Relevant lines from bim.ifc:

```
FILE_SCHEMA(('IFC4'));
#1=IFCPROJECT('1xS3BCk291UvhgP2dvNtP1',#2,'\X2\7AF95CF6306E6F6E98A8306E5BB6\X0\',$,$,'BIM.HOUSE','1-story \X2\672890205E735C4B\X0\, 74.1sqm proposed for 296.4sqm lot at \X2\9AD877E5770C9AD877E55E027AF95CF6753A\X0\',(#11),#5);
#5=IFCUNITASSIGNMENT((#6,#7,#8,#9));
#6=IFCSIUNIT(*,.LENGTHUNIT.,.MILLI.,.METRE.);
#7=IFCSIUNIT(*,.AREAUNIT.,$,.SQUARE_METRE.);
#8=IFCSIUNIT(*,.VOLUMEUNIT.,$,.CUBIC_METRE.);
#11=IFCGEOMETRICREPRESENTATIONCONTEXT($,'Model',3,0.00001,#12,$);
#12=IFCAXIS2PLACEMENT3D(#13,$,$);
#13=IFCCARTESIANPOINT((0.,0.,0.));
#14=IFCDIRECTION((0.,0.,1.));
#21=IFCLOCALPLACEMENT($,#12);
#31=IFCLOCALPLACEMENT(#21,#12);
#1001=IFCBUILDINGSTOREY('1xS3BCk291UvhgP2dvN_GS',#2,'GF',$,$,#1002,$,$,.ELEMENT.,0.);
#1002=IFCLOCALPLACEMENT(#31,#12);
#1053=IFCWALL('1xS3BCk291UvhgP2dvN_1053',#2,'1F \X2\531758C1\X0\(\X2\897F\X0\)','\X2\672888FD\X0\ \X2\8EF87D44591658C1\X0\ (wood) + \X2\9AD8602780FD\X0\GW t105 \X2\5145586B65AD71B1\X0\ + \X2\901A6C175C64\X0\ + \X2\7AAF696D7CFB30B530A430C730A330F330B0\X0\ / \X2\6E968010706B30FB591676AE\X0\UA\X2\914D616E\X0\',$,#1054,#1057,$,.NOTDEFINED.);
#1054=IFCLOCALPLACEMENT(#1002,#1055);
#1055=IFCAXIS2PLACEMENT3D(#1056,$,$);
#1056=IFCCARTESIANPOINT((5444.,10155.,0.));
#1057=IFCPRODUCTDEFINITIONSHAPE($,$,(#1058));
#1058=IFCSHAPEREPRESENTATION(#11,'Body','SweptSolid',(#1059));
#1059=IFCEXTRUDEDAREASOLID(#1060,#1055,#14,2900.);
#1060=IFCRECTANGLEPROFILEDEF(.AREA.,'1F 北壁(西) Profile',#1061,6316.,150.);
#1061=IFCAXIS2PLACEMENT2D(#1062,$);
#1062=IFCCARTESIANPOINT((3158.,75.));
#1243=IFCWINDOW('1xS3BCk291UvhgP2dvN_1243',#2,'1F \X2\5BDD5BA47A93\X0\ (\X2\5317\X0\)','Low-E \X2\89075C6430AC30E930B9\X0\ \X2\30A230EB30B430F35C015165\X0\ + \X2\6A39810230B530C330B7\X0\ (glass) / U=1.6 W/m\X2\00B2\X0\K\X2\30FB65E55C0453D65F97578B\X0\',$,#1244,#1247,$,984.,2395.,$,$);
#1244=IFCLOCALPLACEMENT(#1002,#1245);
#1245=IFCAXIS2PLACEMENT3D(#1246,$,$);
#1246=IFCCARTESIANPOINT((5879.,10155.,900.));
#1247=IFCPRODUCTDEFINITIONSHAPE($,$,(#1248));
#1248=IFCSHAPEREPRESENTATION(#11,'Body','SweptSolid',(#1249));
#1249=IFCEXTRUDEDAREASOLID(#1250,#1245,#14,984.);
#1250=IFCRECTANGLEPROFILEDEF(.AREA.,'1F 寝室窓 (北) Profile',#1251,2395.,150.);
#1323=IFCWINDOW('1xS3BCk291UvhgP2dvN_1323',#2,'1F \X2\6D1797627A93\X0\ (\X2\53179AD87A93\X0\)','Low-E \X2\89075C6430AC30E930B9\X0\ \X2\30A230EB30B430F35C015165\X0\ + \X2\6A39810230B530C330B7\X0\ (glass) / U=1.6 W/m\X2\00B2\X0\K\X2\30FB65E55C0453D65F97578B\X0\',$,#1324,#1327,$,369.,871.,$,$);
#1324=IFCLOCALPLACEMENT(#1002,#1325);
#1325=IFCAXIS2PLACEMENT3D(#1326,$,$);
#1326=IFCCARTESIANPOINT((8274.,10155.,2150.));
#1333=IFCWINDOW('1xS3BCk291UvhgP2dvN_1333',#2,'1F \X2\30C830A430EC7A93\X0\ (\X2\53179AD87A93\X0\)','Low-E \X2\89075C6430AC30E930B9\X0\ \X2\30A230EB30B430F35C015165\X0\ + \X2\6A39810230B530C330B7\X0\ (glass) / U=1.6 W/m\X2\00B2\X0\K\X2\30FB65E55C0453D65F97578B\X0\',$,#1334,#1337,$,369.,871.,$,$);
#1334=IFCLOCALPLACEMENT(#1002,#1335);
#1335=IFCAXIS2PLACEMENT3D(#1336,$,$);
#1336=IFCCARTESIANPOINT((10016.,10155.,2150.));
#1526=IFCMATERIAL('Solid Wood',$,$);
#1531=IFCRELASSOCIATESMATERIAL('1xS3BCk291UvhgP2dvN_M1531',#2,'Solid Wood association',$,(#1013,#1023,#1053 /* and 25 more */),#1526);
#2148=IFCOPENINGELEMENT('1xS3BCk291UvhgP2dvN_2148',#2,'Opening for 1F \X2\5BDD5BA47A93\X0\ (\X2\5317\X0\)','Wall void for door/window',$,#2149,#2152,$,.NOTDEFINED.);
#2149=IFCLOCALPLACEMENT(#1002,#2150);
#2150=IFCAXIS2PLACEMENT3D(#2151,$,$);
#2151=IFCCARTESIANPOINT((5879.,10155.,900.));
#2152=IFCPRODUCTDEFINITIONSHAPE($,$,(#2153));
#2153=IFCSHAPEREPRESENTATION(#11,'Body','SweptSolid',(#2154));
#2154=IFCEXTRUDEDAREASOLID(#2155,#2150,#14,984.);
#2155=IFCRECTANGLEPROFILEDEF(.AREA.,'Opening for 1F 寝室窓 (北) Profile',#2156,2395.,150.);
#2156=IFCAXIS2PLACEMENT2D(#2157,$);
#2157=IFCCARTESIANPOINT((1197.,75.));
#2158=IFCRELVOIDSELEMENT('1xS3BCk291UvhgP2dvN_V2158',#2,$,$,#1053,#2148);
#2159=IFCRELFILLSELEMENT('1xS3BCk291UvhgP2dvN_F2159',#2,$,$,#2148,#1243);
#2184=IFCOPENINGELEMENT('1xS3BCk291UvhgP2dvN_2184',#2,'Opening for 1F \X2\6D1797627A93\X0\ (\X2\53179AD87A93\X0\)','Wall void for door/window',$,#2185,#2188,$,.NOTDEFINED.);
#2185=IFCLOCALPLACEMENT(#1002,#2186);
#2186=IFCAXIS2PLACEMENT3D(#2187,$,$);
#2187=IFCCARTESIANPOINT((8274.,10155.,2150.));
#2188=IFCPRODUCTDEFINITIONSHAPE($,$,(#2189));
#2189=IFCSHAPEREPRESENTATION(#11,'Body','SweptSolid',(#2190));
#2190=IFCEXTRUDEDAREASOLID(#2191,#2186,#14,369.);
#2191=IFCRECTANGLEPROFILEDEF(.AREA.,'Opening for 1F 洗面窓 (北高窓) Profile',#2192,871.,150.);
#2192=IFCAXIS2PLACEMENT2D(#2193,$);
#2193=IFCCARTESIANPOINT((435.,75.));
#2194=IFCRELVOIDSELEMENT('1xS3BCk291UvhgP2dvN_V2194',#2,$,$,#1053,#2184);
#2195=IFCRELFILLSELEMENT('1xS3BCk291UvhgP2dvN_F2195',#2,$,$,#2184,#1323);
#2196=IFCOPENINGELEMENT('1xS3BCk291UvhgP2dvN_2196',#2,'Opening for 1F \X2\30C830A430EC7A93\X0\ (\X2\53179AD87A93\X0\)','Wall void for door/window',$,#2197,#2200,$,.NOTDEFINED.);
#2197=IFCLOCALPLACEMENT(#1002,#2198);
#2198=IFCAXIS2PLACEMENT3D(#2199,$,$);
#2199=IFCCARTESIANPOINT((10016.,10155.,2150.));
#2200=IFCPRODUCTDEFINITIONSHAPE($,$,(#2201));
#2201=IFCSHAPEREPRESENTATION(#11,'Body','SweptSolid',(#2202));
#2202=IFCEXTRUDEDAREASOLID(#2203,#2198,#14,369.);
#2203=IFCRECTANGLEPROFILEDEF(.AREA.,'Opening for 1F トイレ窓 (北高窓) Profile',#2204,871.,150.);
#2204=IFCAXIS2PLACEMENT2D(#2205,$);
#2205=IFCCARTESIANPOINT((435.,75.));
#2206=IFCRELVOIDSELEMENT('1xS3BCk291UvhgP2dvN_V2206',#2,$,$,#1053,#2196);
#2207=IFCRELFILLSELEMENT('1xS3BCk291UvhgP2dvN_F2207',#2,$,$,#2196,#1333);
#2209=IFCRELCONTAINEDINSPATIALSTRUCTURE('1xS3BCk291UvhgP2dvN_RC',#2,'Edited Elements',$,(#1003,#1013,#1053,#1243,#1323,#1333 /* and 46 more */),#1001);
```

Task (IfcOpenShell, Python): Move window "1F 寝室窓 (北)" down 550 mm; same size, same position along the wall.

```python
import numpy as np
import ifcopenshell
import ifcopenshell.api.geometry
import ifcopenshell.util.placement
import ifcopenshell.util.unit

model = ifcopenshell.open("bim.ifc")
unit_scale = ifcopenshell.util.unit.calculate_unit_scale(model)

window = model.by_guid("1xS3BCk291UvhgP2dvN_1243")
opening = window.FillsVoids[0].RelatingOpeningElement
dz = -550.0

shift = np.array([0.0, 0.0, dz])
# The window is not placed relative to its opening, so move both.
for product in (opening, window):
    matrix = ifcopenshell.util.placement.get_local_placement(product.ObjectPlacement)
    matrix[:3, 3] += shift
    ifcopenshell.api.geometry.edit_object_placement(model, product=product, matrix=matrix, is_si=False)

print(f"moved by {dz * unit_scale:+.3f} m")

model.write("bim_v2.ifc")
```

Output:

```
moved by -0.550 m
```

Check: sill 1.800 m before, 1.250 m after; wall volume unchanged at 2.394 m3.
